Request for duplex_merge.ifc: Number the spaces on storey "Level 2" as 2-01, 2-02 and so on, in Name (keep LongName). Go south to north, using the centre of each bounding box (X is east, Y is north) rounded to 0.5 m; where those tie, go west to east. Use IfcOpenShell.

First a look at what the model holds.

```python
import ifcopenshell
import ifcopenshell.util.element
import ifcopenshell.util.placement

model = ifcopenshell.open("duplex_merge.ifc")
print(model.schema)
storey = next(s for s in model.by_type("IfcBuildingStorey") if s.Name == "Level 2")
spaces = [e for e in ifcopenshell.util.element.get_decomposition(storey) if e.is_a("IfcSpace")]
for e in sorted(spaces, key=lambda e: e.id()):
    origin = ifcopenshell.util.placement.get_local_placement(e.ObjectPlacement)[:3, 3]
    print(e.id(), e.Name, e.LongName, origin.round(2) + 0.0, sep=" | ")
```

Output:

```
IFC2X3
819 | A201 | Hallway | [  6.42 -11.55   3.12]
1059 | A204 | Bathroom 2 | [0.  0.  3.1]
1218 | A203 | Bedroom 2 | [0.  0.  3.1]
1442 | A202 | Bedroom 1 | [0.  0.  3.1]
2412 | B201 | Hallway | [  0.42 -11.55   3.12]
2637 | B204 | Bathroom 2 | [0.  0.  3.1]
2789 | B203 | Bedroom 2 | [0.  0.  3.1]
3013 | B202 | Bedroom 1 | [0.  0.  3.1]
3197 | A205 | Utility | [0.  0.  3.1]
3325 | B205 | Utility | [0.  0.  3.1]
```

```python
import ifcopenshell
import ifcopenshell.geom
import ifcopenshell.util.element
import ifcopenshell.util.shape

model = ifcopenshell.open("duplex_merge.ifc")
settings = ifcopenshell.geom.settings()
settings.set("use-world-coords", True)


def centre(element):
    shape = ifcopenshell.geom.create_shape(settings, element)
    return ifcopenshell.util.shape.get_bbox_centroid(shape.geometry)


storey = next(s for s in model.by_type("IfcBuildingStorey") if s.Name == "Level 2")
spaces = [e for e in ifcopenshell.util.element.get_decomposition(storey) if e.is_a("IfcSpace")]

# Insertion points can sit at a corner or the storey origin, so sort by the geometry (in metres).
centres = {e: centre(e) for e in spaces}
spaces.sort(key=lambda e: (round(centres[e][1] / 0.5), centres[e][0]))

for i, e in enumerate(spaces, start=1):
    number = f"2-{i:02d}"
    e.Name = number
    print(e.id(), number)

model.write("duplex_merge_updated.ifc")
```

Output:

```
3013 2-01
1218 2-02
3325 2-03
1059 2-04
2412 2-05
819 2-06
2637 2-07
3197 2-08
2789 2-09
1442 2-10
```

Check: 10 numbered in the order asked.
